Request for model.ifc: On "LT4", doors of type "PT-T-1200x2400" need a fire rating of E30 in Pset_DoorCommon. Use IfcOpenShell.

First a look at what the model holds.

```python
import ifcopenshell
import ifcopenshell.util.element

model = ifcopenshell.open("model.ifc")
print(model.schema)
storey = next(s for s in model.by_type("IfcBuildingStorey") if s.Name == "LT4")
doors = [e for e in ifcopenshell.util.element.get_decomposition(storey) if e.is_a("IfcDoor")]
seen = {}
for e in doors:
    element_type = ifcopenshell.util.element.get_type(e)
    key = (element_type.Name if element_type != e and element_type else None, ifcopenshell.util.element.get_pset(e, "Pset_DoorCommon", "FireRating"))
    seen[key] = seen.get(key, 0) + 1
for (name, value), count in sorted(seen.items(), key=str):
    print(count, "x", name, "|", value)
```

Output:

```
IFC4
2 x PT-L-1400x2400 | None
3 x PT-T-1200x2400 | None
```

```python
import ifcopenshell
import ifcopenshell.api.pset
import ifcopenshell.util.element

model = ifcopenshell.open("model.ifc")

storey = next(s for s in model.by_type("IfcBuildingStorey") if s.Name == "LT4")
doors = [e for e in ifcopenshell.util.element.get_decomposition(storey) if e.is_a("IfcDoor")]

count = 0
for e in doors:
    element_type = ifcopenshell.util.element.get_type(e)
    if element_type in (None, e) or element_type.Name != "PT-T-1200x2400":
        continue
    # add_pset returns the element's existing set when there is one.
    pset = ifcopenshell.api.pset.add_pset(model, product=e, name="Pset_DoorCommon")
    ifcopenshell.api.pset.edit_pset(model, pset=pset, properties={"FireRating": "E30"})
    count += 1

print(count, "doors updated")

model.write("model-out.ifc")
```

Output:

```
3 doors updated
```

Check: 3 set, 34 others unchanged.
